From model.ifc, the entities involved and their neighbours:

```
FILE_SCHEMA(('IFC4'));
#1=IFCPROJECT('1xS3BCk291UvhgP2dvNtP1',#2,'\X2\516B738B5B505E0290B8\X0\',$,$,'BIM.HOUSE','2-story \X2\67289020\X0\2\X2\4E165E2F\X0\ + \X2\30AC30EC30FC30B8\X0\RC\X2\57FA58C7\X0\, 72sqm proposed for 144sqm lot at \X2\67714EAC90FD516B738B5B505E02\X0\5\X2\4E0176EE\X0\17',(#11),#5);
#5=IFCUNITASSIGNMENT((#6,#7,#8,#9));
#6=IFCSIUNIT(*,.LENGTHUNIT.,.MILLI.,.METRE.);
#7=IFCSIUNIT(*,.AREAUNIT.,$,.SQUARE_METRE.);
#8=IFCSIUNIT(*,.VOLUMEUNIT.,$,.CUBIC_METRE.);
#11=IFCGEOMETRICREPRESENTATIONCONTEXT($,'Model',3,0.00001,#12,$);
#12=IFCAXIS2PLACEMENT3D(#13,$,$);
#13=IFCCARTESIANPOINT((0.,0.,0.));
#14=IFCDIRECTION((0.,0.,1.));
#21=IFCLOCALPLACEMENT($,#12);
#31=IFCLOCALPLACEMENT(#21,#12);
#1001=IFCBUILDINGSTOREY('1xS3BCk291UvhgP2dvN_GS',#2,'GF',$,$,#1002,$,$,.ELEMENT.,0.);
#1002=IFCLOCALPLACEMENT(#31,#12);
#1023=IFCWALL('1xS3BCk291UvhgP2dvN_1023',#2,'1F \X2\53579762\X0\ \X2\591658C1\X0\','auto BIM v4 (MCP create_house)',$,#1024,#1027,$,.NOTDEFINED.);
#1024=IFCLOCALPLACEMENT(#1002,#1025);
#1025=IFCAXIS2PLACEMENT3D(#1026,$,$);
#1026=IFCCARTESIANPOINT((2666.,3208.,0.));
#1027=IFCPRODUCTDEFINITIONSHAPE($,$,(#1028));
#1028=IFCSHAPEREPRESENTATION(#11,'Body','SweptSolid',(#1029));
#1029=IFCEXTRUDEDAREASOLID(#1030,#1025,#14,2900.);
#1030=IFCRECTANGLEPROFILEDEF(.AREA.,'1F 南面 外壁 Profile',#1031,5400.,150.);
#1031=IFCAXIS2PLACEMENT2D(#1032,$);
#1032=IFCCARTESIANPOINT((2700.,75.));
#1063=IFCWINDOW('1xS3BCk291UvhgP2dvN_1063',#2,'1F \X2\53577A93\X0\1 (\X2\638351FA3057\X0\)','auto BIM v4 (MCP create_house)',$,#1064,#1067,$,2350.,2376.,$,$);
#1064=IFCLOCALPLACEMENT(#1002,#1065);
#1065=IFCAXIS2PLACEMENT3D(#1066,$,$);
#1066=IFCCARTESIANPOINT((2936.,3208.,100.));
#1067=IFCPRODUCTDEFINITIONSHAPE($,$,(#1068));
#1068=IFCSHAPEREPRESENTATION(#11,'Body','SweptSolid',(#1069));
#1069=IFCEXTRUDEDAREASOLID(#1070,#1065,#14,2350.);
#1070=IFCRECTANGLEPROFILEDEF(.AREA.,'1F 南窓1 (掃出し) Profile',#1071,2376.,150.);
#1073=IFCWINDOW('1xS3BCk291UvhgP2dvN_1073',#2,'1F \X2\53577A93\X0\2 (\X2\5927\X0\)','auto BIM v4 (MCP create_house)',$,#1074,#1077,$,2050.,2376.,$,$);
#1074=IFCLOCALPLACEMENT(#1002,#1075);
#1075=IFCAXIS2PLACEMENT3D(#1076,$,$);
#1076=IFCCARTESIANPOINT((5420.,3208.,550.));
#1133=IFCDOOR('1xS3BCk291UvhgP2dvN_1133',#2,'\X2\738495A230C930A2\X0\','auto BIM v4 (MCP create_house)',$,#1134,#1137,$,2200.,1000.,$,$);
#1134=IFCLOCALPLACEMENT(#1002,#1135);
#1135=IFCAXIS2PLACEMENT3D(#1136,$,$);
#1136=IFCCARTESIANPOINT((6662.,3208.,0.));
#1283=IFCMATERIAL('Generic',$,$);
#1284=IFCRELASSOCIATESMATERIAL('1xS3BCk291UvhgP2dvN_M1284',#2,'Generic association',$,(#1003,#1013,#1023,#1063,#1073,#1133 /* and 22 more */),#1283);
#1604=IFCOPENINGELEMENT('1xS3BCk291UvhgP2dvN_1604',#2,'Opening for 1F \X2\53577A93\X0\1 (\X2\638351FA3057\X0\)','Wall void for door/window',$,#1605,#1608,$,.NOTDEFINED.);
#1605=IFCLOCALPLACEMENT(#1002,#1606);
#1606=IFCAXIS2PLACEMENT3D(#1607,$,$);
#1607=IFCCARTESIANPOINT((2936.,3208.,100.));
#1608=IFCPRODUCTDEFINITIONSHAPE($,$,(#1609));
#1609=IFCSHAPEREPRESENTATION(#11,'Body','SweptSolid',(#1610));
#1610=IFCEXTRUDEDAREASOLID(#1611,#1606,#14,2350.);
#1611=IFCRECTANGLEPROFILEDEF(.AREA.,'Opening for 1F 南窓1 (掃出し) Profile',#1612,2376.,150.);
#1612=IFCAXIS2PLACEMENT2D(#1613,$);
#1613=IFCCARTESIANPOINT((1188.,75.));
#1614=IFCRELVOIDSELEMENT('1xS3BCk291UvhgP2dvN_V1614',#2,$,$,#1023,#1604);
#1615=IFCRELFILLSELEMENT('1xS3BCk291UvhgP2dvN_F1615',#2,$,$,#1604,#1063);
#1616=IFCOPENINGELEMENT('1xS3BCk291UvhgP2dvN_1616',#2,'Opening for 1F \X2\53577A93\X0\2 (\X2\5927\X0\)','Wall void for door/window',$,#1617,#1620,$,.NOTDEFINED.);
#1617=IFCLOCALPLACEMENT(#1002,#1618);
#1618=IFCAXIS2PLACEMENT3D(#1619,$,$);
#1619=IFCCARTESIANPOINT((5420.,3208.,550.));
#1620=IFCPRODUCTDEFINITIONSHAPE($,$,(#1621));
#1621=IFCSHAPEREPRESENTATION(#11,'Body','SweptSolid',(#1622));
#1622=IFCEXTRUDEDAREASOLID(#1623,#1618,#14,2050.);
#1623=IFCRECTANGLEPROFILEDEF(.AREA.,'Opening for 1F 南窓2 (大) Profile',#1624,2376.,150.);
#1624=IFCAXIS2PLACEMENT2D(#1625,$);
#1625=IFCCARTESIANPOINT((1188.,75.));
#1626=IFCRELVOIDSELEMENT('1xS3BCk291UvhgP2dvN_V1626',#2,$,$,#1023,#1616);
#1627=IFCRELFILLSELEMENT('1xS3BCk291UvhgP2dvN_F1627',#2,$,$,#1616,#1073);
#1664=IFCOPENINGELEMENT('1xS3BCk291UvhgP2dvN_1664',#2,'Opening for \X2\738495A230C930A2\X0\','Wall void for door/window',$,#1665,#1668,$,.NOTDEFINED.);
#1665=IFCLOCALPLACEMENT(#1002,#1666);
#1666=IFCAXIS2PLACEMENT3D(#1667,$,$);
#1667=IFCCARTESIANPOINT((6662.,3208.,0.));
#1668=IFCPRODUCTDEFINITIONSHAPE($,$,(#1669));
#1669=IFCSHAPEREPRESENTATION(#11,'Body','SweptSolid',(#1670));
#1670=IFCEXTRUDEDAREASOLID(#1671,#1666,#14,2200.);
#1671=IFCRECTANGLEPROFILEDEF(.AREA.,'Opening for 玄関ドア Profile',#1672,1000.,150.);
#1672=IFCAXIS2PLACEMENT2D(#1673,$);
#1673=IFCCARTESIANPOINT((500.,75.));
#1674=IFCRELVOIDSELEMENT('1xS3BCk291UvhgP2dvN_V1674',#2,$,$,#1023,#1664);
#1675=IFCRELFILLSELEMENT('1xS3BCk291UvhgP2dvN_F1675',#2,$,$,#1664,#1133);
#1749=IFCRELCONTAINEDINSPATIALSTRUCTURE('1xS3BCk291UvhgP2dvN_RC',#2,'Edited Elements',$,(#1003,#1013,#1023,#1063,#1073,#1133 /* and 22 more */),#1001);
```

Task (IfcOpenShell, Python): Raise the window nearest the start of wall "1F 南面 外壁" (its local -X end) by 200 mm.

```python
import numpy as np
import ifcopenshell
import ifcopenshell.api.geometry
import ifcopenshell.util.placement
import ifcopenshell.util.unit

model = ifcopenshell.open("model.ifc")
unit_scale = ifcopenshell.util.unit.calculate_unit_scale(model)

window = model.by_id(1063)
opening = window.FillsVoids[0].RelatingOpeningElement
dz = 200.0

shift = np.array([0.0, 0.0, dz])
# The window is not placed relative to its opening, so move both.
for product in (opening, window):
    matrix = ifcopenshell.util.placement.get_local_placement(product.ObjectPlacement)
    matrix[:3, 3] += shift
    ifcopenshell.api.geometry.edit_object_placement(model, product=product, matrix=matrix, is_si=False)

print(f"moved by {dz * unit_scale:+.3f} m")

model.write("model_v2.ifc")
```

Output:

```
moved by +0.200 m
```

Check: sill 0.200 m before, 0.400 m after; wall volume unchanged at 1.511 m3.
